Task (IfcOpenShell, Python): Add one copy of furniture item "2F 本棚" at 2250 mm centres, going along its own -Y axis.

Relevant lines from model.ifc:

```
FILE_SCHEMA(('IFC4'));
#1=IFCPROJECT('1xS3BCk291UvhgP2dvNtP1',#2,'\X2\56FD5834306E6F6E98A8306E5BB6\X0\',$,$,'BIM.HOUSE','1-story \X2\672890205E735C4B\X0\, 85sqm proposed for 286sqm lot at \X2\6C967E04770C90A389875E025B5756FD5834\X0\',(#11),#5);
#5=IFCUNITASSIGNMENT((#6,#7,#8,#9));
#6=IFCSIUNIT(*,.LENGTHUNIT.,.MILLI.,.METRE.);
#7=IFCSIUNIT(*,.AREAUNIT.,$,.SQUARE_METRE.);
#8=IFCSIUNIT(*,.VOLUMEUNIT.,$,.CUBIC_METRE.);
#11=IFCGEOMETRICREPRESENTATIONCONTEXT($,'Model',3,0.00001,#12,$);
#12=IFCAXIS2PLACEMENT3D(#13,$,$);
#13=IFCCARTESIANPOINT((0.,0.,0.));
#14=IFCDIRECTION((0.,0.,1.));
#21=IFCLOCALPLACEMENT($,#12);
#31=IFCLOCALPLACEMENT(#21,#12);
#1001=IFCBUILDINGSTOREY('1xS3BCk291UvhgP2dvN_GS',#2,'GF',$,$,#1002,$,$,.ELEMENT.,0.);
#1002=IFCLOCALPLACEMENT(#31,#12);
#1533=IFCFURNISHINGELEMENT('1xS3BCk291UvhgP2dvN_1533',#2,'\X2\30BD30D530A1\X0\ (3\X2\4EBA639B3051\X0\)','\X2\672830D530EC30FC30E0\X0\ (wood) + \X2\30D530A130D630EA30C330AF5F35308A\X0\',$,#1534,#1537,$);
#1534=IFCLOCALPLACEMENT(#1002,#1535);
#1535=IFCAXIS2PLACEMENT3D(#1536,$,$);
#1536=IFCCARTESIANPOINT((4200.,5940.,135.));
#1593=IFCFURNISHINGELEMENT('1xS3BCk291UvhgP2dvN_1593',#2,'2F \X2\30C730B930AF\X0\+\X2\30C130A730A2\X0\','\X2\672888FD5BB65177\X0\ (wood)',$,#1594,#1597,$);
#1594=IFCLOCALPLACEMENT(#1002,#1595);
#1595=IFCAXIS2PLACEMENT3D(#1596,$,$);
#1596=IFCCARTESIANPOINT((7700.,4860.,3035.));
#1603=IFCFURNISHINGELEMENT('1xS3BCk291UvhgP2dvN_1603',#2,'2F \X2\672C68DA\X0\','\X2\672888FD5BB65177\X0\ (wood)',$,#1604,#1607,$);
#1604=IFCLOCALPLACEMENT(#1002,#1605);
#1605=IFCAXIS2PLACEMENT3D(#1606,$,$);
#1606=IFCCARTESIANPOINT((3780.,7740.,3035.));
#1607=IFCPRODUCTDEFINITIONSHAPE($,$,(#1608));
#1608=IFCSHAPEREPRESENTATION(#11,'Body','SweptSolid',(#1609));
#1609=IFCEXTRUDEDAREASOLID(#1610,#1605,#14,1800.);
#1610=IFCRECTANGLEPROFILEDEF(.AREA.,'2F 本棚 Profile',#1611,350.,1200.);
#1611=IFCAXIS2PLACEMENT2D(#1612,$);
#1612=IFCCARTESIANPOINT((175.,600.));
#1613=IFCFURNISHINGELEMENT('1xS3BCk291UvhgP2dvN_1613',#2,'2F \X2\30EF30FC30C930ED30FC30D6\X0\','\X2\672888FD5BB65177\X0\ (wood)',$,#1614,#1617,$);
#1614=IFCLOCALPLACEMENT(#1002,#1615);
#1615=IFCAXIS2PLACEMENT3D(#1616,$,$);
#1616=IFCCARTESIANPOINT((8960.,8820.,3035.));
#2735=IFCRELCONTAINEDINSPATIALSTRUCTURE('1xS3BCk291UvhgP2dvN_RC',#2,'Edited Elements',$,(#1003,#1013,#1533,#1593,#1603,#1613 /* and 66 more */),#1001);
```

```python
import ifcopenshell
import ifcopenshell.api.geometry
import ifcopenshell.api.root
import ifcopenshell.util.element
import ifcopenshell.util.placement
import ifcopenshell.util.unit

model = ifcopenshell.open("model.ifc")
unit_scale = ifcopenshell.util.unit.calculate_unit_scale(model)


def reuse_history(source, copy):
    """copy_class also copies each property set's owner history, people and application; keep the originals."""
    for rel in copy.IsDefinedBy:
        if rel.is_a("IfcRelDefinesByProperties") and (history := rel.RelatingPropertyDefinition.OwnerHistory):
            rel.RelatingPropertyDefinition.OwnerHistory = source.OwnerHistory
            ifcopenshell.util.element.remove_deep2(model, history)


source = model.by_id(1603)
base = ifcopenshell.util.placement.get_local_placement(source.ObjectPlacement)
step = -base[:3, 1] * 2.25 / unit_scale

for i in range(1, 2):
    copy = ifcopenshell.api.root.copy_class(model, product=source)
    copy.Representation = ifcopenshell.util.element.copy_deep(
        model, source.Representation, exclude=["IfcGeometricRepresentationContext", "IfcRepresentationMap"]
    )
    reuse_history(source, copy)
    matrix = base.copy()
    matrix[:3, 3] += i * step
    print("added at", matrix[:3, 3].round(3) + 0.0)
    ifcopenshell.api.geometry.edit_object_placement(model, product=copy, matrix=matrix, is_si=False)

model.write("model_rev.ifc")
```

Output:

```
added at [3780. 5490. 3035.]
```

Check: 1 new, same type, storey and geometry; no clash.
